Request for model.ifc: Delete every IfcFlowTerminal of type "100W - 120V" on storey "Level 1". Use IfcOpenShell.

First a look at what the model holds.

```python
import ifcopenshell
import ifcopenshell.util.element

model = ifcopenshell.open("model.ifc")
print(model.schema)
storey = next(s for s in model.by_type("IfcBuildingStorey") if s.Name == "Level 1")
terminals = [e for e in ifcopenshell.util.element.get_decomposition(storey) if e.is_a("IfcFlowTerminal")]
seen = {}
for e in terminals:
    element_type = ifcopenshell.util.element.get_type(e)
    name = element_type.Name if element_type not in (None, e) else None
    seen[name] = seen.get(name, 0) + 1
for name, count in sorted(seen.items(), key=str):
    print(count, "x", name)
```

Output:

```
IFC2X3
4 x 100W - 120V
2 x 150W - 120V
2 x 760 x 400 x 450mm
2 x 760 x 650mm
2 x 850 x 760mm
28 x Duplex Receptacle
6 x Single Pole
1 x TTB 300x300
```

```python
import ifcopenshell
import ifcopenshell.api.root
import ifcopenshell.util.element

model = ifcopenshell.open("model.ifc")

storey = next(s for s in model.by_type("IfcBuildingStorey") if s.Name == "Level 1")
terminals = [e for e in ifcopenshell.util.element.get_decomposition(storey) if e.is_a("IfcFlowTerminal")]
targets = [e for e in terminals if (t := ifcopenshell.util.element.get_type(e)) not in (None, e) and t.Name == "100W - 120V"]

for e in targets:
    ifcopenshell.api.root.remove_product(model, product=e)
print(len(targets), "removed")

model.write("model_v2.ifc")
```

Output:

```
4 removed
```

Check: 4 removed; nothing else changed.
